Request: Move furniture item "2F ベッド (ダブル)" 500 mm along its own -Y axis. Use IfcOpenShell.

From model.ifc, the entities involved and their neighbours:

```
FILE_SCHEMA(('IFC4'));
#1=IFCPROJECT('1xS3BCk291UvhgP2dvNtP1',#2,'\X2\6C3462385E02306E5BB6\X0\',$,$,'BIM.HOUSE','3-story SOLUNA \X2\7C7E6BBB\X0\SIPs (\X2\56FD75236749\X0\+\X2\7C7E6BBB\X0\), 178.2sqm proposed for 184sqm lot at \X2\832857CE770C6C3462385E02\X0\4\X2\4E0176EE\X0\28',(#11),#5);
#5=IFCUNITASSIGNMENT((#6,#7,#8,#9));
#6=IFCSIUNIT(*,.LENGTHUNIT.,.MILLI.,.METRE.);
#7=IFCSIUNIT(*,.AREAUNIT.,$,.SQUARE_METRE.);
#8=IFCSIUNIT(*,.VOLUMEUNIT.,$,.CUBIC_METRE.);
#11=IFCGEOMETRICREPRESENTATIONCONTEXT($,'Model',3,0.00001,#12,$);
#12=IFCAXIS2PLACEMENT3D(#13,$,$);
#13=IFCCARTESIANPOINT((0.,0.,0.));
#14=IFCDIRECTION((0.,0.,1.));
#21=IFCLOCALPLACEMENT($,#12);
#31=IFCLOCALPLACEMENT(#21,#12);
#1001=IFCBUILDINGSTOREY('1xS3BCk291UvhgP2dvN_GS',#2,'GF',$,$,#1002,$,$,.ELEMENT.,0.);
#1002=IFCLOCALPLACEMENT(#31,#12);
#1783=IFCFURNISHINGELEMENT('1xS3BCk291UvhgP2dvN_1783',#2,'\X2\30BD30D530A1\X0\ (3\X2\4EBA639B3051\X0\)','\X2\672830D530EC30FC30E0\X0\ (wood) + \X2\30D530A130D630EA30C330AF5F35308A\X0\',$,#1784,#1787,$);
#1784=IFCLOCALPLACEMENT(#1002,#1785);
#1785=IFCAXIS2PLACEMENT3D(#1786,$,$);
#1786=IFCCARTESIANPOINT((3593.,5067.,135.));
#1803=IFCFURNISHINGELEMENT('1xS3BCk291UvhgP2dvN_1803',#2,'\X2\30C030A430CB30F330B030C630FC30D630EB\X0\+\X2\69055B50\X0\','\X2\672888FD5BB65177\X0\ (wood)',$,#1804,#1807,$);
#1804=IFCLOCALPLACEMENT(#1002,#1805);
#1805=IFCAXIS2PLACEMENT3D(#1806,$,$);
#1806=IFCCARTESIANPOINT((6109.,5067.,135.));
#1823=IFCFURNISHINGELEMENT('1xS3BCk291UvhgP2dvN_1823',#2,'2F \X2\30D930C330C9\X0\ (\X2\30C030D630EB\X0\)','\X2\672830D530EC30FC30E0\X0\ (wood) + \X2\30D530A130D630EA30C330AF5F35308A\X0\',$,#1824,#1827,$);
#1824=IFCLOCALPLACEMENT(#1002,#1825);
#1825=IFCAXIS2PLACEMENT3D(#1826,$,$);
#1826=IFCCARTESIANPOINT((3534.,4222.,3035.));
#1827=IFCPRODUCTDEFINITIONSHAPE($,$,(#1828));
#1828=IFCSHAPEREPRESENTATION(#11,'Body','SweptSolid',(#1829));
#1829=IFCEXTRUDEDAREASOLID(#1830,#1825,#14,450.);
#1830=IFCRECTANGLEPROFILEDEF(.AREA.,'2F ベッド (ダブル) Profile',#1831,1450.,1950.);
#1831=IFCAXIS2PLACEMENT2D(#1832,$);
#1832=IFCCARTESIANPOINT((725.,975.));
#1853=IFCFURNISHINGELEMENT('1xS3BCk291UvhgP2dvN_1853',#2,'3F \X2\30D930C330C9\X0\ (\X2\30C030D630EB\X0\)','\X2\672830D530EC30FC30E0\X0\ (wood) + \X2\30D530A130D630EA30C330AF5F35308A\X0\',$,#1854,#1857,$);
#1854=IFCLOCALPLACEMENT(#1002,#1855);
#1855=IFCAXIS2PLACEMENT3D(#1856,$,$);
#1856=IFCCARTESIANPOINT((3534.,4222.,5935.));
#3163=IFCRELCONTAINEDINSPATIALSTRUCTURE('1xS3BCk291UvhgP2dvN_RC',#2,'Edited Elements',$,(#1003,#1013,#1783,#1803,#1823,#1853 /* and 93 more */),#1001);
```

```python
import ifcopenshell
import ifcopenshell.api.geometry
import ifcopenshell.util.placement
import ifcopenshell.util.unit

model = ifcopenshell.open("model.ifc")
unit_scale = ifcopenshell.util.unit.calculate_unit_scale(model)

item = model.by_guid("1xS3BCk291UvhgP2dvN_1823")
matrix = ifcopenshell.util.placement.get_local_placement(item.ObjectPlacement)
matrix[:3, 3] -= matrix[:3, 1] * 0.5 / unit_scale
ifcopenshell.api.geometry.edit_object_placement(model, product=item, matrix=matrix, is_si=False)

print(ifcopenshell.util.placement.get_local_placement(item.ObjectPlacement).round(3) + 0.0)

model.write("model_updated.ifc")
```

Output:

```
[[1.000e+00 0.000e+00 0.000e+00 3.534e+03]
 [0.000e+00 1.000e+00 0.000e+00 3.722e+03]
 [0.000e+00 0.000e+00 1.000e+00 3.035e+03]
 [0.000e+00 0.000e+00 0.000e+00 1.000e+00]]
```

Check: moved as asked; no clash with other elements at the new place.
